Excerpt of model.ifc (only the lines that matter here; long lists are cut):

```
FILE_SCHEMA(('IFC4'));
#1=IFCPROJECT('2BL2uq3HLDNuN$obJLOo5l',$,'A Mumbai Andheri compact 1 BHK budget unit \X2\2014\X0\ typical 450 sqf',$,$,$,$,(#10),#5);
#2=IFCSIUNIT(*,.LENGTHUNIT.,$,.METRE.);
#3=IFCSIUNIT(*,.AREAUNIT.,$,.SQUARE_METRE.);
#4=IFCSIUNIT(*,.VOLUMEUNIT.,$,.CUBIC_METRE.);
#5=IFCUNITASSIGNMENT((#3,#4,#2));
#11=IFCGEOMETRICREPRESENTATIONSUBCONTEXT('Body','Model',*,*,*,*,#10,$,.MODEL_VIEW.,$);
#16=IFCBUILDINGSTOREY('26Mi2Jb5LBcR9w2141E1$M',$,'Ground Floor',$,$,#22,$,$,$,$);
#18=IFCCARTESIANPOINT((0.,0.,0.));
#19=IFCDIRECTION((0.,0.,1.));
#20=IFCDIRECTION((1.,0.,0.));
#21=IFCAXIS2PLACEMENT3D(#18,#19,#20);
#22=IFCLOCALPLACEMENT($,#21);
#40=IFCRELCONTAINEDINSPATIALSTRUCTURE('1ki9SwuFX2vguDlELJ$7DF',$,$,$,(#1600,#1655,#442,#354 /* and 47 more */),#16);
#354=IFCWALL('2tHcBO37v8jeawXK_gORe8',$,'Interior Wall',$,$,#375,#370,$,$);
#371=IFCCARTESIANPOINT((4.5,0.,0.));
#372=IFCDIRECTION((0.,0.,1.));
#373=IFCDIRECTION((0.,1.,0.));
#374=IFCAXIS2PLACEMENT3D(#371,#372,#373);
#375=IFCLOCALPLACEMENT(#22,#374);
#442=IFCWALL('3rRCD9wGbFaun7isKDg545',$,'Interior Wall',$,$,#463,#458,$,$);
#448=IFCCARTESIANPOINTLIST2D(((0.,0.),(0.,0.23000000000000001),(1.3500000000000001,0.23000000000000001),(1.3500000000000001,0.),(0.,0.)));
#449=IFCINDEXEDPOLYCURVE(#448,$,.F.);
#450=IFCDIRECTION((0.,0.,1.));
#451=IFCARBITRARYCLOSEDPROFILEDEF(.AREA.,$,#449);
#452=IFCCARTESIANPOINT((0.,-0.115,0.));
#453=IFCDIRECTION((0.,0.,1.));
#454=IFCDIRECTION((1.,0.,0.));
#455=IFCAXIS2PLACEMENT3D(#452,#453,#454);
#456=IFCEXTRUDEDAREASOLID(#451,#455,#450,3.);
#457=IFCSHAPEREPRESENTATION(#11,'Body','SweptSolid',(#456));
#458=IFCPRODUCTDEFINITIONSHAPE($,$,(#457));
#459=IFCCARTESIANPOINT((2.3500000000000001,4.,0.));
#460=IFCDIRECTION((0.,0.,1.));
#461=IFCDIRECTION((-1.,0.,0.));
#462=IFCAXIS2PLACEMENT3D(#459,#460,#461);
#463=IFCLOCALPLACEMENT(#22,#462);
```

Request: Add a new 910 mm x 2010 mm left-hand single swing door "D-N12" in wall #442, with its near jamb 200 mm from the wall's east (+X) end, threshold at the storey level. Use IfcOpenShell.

```python
import numpy as np
import ifcopenshell
import ifcopenshell.api.feature
import ifcopenshell.api.geometry
import ifcopenshell.api.root
import ifcopenshell.api.spatial
import ifcopenshell.geom
import ifcopenshell.util.element
import ifcopenshell.util.placement
import ifcopenshell.util.representation
import ifcopenshell.util.shape
import ifcopenshell.util.unit

model = ifcopenshell.open("model.ifc")
unit_scale = ifcopenshell.util.unit.calculate_unit_scale(model)
settings = ifcopenshell.geom.settings()


def volume(element):
    """Net volume in cubic metres, openings subtracted."""
    shape = ifcopenshell.geom.create_shape(settings, element)
    return ifcopenshell.util.shape.get_volume(shape.geometry)


wall = model.by_guid("3rRCD9wGbFaun7isKDg545")
storey = ifcopenshell.util.element.get_container(wall, ifc_class="IfcBuildingStorey")
context = ifcopenshell.util.representation.get_context(model, "Model", "Body", "MODEL_VIEW")
before = volume(wall)

width, height, from_end, sill = 0.91, 2.01, 0.2, 0.0  # metres

# The wall runs along its own X axis, and the end named is its -X end.
wall_shape = ifcopenshell.geom.create_shape(settings, wall)
x, y, z = ifcopenshell.util.shape.get_vertices(wall_shape.geometry).T
start = x.min() + from_end
face, thickness = float(y.min()), float(y.max() - y.min())
wall_matrix = ifcopenshell.util.placement.get_local_placement(wall.ObjectPlacement)
level = ifcopenshell.util.placement.get_local_placement(storey.ObjectPlacement)[2, 3]


def in_wall(x, y):
    """Placement at x, y metres in the wall's axes, at sill height."""
    matrix = wall_matrix.copy()
    matrix[:, 3] = wall_matrix @ np.array([x / unit_scale, y / unit_scale, 0.0, 1.0])
    matrix[2, 3] = level + sill / unit_scale
    return matrix


# Opening: a box that overshoots both wall faces by 50 mm.
opening = ifcopenshell.api.root.create_entity(model, ifc_class="IfcOpeningElement", predefined_type="OPENING")
box = ifcopenshell.api.geometry.add_wall_representation(
    model, context=context, length=width, height=height, thickness=thickness + 0.1
)
ifcopenshell.api.geometry.assign_representation(model, product=opening, representation=box)
ifcopenshell.api.geometry.edit_object_placement(model, product=opening, matrix=in_wall(start, face - 0.05), is_si=False)
ifcopenshell.api.feature.add_feature(model, feature=opening, element=wall)

door = ifcopenshell.api.root.create_entity(model, ifc_class="IfcDoor", name="D-N12", predefined_type="DOOR")
door.OverallWidth, door.OverallHeight = width / unit_scale, height / unit_scale
door.OperationType = "SINGLE_SWING_LEFT"
body = ifcopenshell.api.geometry.add_door_representation(
    model,
    context=context,
    overall_width=door.OverallWidth,
    overall_height=door.OverallHeight,
    operation_type="SINGLE_SWING_LEFT",
    lining_properties={"LiningDepth": thickness / unit_scale, "ThresholdDepth": thickness / unit_scale},
)
ifcopenshell.api.geometry.assign_representation(model, product=door, representation=body)
ifcopenshell.api.spatial.assign_container(model, products=[door], relating_structure=storey)
ifcopenshell.api.feature.add_filling(model, opening=opening, element=door)

# The lining spans the wall, so the door starts at the wall face.
ifcopenshell.api.geometry.edit_object_placement(model, product=door, matrix=in_wall(start, face), is_si=False)

after = volume(wall)

print(f"wall volume {before:.3f} -> {after:.3f} m3")

model.write("model_v2.ifc")
```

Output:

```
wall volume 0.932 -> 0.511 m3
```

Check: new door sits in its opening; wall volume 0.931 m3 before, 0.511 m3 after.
